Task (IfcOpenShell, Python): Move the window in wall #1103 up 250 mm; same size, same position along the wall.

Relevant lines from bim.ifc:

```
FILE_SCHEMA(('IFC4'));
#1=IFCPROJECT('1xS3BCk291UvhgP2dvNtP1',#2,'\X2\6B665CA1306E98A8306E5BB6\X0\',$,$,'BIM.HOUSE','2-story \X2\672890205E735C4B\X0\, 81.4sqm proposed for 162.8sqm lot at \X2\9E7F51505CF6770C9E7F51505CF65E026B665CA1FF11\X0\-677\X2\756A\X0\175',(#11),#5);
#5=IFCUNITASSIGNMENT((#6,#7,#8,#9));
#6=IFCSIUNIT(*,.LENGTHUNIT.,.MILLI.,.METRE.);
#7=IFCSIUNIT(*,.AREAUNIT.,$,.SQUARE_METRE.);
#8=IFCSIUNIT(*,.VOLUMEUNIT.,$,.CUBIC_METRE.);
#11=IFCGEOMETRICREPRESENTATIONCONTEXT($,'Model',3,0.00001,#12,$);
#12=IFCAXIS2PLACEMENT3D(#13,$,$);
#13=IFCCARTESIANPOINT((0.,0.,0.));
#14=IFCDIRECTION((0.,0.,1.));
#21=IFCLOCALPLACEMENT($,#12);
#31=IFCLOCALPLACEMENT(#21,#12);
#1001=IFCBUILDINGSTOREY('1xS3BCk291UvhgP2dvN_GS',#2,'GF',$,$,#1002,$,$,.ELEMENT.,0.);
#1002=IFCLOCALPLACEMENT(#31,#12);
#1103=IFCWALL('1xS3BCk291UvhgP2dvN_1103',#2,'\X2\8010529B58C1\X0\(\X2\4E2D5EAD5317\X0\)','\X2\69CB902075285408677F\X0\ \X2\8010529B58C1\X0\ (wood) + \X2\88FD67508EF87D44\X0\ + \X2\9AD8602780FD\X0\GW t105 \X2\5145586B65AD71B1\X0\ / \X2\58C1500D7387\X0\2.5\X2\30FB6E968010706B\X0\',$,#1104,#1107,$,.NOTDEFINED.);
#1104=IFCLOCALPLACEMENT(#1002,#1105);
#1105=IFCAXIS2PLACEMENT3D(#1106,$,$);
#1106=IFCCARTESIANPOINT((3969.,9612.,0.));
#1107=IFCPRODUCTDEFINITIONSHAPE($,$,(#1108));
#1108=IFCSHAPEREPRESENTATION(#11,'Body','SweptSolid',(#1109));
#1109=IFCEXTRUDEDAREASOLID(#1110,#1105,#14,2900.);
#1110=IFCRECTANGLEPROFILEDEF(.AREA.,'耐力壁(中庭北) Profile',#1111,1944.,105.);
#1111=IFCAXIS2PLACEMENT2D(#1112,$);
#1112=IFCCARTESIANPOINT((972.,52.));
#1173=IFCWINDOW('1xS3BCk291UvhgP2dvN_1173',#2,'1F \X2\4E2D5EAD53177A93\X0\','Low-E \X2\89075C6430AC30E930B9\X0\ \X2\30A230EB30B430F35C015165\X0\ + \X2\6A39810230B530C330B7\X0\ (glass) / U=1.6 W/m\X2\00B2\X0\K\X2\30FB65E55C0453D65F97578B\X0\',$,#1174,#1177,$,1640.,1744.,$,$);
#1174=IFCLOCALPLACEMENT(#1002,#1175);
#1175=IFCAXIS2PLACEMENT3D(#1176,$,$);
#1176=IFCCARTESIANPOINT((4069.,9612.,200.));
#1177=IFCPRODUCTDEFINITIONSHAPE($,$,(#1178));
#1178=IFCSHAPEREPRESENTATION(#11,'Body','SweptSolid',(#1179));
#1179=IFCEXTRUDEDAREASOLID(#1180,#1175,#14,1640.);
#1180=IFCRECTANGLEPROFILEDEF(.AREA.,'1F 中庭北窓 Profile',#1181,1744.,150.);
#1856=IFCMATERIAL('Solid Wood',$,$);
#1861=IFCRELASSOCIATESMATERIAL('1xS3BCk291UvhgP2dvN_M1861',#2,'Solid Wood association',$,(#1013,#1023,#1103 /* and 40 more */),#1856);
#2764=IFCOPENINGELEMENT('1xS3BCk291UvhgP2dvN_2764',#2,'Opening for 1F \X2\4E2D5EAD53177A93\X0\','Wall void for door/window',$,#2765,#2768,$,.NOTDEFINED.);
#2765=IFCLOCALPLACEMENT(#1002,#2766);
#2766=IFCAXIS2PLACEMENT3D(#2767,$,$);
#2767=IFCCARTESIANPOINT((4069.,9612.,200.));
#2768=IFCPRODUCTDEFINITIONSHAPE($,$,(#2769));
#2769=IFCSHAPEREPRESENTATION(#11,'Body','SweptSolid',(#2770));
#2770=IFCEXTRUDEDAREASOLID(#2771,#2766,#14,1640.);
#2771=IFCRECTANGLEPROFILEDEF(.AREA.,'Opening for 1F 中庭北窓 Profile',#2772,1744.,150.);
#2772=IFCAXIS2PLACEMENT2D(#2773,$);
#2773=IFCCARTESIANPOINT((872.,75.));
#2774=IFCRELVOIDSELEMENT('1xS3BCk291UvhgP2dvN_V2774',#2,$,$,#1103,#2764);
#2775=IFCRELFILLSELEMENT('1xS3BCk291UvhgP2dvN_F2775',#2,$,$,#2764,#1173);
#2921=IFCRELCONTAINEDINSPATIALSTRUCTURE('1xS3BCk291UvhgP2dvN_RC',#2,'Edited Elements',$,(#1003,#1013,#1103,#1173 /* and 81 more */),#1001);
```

```python
import numpy as np
import ifcopenshell
import ifcopenshell.api.geometry
import ifcopenshell.util.placement
import ifcopenshell.util.unit

model = ifcopenshell.open("bim.ifc")
unit_scale = ifcopenshell.util.unit.calculate_unit_scale(model)

window = model.by_guid("1xS3BCk291UvhgP2dvN_1173")
opening = window.FillsVoids[0].RelatingOpeningElement
dz = 250.0

shift = np.array([0.0, 0.0, dz])
# The window is not placed relative to its opening, so move both.
for product in (opening, window):
    matrix = ifcopenshell.util.placement.get_local_placement(product.ObjectPlacement)
    matrix[:3, 3] += shift
    ifcopenshell.api.geometry.edit_object_placement(model, product=product, matrix=matrix, is_si=False)

print(f"moved by {dz * unit_scale:+.3f} m")

model.write("bim-out.ifc")
```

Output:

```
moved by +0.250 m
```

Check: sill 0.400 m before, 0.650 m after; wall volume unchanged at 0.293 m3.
